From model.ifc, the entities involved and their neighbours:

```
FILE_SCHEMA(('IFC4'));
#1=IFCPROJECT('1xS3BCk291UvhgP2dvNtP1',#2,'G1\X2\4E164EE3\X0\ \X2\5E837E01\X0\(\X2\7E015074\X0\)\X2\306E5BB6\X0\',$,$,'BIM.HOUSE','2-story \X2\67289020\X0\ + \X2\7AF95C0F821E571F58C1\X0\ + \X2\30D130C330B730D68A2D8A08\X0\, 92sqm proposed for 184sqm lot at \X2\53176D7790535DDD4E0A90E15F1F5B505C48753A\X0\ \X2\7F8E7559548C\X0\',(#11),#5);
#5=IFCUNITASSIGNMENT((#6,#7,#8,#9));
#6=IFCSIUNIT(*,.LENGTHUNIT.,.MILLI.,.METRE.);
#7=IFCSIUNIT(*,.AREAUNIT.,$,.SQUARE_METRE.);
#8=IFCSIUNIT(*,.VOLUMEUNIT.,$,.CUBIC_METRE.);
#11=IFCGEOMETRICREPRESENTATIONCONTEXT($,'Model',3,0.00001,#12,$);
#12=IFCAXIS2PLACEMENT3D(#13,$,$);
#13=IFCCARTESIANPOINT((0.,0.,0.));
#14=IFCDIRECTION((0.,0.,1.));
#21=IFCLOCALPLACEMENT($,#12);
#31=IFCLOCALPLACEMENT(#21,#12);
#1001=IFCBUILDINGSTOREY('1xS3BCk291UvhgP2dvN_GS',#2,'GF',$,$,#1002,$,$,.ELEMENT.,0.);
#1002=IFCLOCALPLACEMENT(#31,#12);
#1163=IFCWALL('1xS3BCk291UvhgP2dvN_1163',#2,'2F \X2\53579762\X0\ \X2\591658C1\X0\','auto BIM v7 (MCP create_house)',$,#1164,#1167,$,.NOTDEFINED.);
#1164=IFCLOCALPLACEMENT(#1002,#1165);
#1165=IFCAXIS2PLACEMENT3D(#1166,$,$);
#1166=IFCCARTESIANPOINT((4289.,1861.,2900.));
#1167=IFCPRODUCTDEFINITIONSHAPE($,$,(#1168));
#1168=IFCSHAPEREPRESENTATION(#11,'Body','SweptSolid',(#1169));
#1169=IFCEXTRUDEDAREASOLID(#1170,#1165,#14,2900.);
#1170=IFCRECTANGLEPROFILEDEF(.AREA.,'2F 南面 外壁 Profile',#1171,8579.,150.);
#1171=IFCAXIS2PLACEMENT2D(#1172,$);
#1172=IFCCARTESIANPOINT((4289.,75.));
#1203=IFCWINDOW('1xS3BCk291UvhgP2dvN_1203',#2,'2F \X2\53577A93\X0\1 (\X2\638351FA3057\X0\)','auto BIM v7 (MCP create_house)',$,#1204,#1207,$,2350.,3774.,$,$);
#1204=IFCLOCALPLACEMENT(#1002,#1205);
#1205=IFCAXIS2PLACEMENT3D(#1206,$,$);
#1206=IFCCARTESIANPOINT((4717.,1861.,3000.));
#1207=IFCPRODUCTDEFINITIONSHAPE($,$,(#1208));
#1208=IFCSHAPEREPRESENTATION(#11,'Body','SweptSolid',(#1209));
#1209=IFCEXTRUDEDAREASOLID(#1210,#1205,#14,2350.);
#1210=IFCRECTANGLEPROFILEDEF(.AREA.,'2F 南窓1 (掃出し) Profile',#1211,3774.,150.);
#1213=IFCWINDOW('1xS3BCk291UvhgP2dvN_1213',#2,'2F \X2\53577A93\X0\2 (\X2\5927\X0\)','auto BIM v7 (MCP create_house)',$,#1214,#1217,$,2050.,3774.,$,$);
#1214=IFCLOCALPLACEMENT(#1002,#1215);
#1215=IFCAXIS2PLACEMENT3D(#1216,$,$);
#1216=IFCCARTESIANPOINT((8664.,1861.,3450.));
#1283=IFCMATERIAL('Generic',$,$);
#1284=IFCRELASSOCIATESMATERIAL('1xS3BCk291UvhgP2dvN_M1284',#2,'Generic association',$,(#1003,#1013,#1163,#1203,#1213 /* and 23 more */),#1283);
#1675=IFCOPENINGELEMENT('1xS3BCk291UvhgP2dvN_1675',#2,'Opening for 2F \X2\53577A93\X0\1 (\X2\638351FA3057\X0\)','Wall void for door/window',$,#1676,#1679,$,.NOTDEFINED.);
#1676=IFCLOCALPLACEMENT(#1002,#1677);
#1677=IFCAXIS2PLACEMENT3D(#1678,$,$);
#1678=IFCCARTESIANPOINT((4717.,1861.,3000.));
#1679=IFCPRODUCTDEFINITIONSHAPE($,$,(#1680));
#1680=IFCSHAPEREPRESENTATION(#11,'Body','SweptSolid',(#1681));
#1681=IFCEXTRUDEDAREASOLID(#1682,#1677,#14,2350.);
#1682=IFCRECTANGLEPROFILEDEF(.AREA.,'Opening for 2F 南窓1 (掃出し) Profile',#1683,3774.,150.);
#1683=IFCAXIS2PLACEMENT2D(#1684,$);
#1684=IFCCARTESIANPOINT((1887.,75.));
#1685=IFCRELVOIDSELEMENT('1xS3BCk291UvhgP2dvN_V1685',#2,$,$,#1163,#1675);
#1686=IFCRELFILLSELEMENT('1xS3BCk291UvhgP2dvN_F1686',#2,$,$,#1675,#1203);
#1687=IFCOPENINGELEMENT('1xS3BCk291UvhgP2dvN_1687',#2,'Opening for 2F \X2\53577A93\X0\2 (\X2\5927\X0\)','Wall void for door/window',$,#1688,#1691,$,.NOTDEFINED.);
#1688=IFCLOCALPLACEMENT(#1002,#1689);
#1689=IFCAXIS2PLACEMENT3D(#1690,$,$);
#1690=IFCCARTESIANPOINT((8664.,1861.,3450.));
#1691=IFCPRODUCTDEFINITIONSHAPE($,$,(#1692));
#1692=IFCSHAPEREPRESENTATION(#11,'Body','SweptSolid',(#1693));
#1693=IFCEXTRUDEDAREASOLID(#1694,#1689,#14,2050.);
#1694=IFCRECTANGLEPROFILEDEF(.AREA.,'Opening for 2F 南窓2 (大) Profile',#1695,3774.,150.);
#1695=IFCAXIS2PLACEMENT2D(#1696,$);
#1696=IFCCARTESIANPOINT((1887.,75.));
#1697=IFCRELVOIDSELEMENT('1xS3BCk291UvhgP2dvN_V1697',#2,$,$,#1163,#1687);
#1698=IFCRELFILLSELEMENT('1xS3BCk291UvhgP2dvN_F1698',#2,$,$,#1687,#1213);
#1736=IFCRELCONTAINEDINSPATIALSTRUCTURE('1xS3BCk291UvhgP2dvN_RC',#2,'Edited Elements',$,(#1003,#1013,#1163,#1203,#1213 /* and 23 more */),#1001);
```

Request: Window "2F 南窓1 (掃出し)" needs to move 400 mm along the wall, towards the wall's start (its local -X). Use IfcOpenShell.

```python
import ifcopenshell
import ifcopenshell.api.geometry
import ifcopenshell.util.placement

model = ifcopenshell.open("model.ifc")

window = model.by_id(1203)
opening = window.FillsVoids[0].RelatingOpeningElement
wall = opening.VoidsElements[0].RelatingBuildingElement

wall_matrix = ifcopenshell.util.placement.get_local_placement(wall.ObjectPlacement)
shift = wall_matrix[:3, 0] * -400.0
before = ifcopenshell.util.placement.get_local_placement(window.ObjectPlacement)[:3, 3].copy()

# The window is not placed relative to its opening, so move both.
for product in (opening, window):
    matrix = ifcopenshell.util.placement.get_local_placement(product.ObjectPlacement)
    matrix[:3, 3] += shift
    ifcopenshell.api.geometry.edit_object_placement(model, product=product, matrix=matrix, is_si=False)

after = ifcopenshell.util.placement.get_local_placement(window.ObjectPlacement)[:3, 3]
print("window moved by", (after - before).round(3) + 0.0)

model.write("model-out.ifc")
```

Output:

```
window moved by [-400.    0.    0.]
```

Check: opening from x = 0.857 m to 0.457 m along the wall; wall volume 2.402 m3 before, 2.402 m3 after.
